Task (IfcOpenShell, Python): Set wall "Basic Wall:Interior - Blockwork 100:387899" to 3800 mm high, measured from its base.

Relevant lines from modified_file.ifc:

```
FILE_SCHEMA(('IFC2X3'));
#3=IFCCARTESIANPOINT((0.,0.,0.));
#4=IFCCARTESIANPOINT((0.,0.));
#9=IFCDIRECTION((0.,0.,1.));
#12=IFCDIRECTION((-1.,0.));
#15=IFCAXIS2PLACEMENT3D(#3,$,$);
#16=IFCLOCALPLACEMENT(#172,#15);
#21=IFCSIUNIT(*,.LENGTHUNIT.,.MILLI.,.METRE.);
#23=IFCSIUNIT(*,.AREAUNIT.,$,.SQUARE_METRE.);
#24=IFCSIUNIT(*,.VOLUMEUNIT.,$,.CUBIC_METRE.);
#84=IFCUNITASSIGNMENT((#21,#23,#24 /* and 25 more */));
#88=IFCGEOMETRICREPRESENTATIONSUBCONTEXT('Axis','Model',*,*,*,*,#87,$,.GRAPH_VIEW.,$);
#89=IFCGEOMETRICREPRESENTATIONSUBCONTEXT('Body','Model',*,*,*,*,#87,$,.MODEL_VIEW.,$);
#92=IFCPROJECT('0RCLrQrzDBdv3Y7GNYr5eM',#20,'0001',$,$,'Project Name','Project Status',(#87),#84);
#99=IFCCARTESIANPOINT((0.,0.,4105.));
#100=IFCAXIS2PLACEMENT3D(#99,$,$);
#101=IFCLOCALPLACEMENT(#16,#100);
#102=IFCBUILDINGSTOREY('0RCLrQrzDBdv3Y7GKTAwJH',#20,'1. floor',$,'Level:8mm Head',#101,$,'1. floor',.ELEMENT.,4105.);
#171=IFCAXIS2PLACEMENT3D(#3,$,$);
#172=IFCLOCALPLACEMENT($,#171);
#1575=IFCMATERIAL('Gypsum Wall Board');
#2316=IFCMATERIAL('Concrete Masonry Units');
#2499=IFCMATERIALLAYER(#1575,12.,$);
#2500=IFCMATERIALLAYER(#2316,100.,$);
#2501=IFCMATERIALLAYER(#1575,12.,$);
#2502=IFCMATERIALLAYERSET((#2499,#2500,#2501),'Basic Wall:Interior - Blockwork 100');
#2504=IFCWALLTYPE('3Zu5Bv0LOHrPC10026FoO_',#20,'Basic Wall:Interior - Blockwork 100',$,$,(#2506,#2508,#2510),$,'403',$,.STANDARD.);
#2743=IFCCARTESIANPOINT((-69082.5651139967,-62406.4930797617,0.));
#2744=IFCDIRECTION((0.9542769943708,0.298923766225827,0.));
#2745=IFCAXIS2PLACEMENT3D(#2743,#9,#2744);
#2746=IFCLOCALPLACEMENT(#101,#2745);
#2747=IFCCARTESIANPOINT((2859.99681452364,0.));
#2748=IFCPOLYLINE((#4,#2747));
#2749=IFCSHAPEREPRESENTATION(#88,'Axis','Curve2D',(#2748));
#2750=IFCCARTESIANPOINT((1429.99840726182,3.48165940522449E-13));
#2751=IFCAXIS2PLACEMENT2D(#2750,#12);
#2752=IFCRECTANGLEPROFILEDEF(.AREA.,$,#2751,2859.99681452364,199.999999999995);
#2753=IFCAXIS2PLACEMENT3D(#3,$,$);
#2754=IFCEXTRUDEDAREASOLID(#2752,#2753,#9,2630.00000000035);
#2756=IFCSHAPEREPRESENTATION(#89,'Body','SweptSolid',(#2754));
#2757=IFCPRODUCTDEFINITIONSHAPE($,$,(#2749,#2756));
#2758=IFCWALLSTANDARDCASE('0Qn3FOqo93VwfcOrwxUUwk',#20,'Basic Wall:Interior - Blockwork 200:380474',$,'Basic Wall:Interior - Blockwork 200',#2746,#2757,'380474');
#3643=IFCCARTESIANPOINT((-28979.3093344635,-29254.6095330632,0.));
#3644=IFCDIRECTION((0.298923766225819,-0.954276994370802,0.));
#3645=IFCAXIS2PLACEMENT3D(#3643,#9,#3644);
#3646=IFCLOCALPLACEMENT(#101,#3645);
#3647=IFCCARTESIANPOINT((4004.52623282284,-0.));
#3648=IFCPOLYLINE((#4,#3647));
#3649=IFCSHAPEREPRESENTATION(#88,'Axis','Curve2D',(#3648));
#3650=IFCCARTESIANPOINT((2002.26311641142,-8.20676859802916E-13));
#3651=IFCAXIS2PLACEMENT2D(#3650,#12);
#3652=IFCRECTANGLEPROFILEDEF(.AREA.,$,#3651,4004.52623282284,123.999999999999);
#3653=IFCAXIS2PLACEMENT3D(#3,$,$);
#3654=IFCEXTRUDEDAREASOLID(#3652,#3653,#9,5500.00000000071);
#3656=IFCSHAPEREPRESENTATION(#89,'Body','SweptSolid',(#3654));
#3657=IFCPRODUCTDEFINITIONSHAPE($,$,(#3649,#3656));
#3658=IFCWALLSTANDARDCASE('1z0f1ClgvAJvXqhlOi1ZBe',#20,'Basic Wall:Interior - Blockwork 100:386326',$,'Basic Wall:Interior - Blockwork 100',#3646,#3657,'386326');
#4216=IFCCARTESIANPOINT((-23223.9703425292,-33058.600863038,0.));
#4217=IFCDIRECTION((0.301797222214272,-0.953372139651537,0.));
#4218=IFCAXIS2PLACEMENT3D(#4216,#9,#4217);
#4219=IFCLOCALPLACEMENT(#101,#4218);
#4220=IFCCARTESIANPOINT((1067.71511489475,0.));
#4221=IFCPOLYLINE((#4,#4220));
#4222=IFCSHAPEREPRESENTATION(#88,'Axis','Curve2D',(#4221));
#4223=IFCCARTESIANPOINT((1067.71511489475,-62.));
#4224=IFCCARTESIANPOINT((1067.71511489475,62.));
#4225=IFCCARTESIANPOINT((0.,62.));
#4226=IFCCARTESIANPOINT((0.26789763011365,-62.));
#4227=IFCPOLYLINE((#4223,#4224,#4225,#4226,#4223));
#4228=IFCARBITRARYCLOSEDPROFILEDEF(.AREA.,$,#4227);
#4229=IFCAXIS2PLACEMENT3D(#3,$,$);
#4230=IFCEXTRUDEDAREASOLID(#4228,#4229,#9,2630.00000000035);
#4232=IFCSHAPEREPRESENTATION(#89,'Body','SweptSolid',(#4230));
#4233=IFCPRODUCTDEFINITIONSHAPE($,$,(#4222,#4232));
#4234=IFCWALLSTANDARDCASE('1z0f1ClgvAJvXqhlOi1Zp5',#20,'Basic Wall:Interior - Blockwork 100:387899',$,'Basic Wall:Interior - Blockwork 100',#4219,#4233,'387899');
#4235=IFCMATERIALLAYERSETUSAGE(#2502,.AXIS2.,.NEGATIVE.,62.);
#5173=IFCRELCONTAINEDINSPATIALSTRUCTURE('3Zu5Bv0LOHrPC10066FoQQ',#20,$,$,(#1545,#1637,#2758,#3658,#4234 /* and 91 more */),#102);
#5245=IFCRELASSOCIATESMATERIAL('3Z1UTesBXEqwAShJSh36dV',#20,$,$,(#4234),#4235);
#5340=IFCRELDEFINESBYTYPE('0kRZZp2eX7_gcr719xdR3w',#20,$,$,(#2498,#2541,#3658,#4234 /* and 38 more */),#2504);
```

```python
import ifcopenshell
import ifcopenshell.geom
import ifcopenshell.util.representation
import ifcopenshell.util.shape
import ifcopenshell.util.unit

model = ifcopenshell.open("modified_file.ifc")
unit_scale = ifcopenshell.util.unit.calculate_unit_scale(model)
settings = ifcopenshell.geom.settings()


def volume(element):
    """Net volume in cubic metres, openings subtracted."""
    shape = ifcopenshell.geom.create_shape(settings, element)
    return ifcopenshell.util.shape.get_volume(shape.geometry)


wall = model.by_guid("1z0f1ClgvAJvXqhlOi1Zp5")
before = volume(wall)

body = ifcopenshell.util.representation.get_representation(wall, "Model", "Body")
solid = body.Items[0]
old_height = solid.Depth
solid.Depth = 3.8 / unit_scale
after = volume(wall)

print(f"height {old_height:g} -> {solid.Depth:g}, volume {before:.3f} -> {after:.3f} m3")

model.write("modified_file_v2.ifc")
```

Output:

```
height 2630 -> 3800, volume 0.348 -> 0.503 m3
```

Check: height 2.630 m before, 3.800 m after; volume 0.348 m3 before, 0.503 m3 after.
